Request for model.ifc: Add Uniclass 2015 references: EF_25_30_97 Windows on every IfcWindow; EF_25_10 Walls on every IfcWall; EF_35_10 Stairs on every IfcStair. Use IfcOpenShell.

First a look at what the model holds.

```python
import ifcopenshell

model = ifcopenshell.open("model.ifc")
print(model.schema)
print("classifications:", [c.Name for c in model.by_type("IfcClassification")])
for ifc_class in ("IfcDoor", "IfcRoof", "IfcStair", "IfcWall", "IfcWindow"):
    print(ifc_class, len(model.by_type(ifc_class)))
```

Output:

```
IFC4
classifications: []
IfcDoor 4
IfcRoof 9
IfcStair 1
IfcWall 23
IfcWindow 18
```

```python
import ifcopenshell
import ifcopenshell.api.classification

model = ifcopenshell.open("model.ifc")

system = ifcopenshell.api.classification.add_classification(model, classification="Uniclass 2015")

codes = {
    "IfcWindow": ("EF_25_30_97", "Windows"),
    "IfcWall": ("EF_25_10", "Walls"),
    "IfcStair": ("EF_35_10", "Stairs"),
}
for ifc_class, (code, name) in codes.items():
    products = model.by_type(ifc_class)
    ifcopenshell.api.classification.add_reference(
        model, products=products, classification=system, identification=code, name=name
    )
    print(code, len(products))

model.write("model_v2.ifc")
```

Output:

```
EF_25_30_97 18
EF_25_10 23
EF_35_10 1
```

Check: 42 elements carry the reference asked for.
